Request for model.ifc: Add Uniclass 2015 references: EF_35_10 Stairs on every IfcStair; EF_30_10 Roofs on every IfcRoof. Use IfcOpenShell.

First a look at what the model holds.

```python
import ifcopenshell

model = ifcopenshell.open("model.ifc")
print(model.schema)
print("classifications:", [c.Name for c in model.by_type("IfcClassification")])
for ifc_class in ("IfcDoor", "IfcRoof", "IfcStair", "IfcWall", "IfcWindow"):
    print(ifc_class, len(model.by_type(ifc_class)))
```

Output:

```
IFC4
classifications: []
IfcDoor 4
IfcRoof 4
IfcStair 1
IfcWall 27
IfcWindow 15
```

```python
import ifcopenshell
import ifcopenshell.api.classification

model = ifcopenshell.open("model.ifc")

system = ifcopenshell.api.classification.add_classification(model, classification="Uniclass 2015")

codes = {
    "IfcStair": ("EF_35_10", "Stairs"),
    "IfcRoof": ("EF_30_10", "Roofs"),
}
for ifc_class, (code, name) in codes.items():
    products = model.by_type(ifc_class)
    ifcopenshell.api.classification.add_reference(
        model, products=products, classification=system, identification=code, name=name
    )
    print(code, len(products))

model.write("model_rev.ifc")
```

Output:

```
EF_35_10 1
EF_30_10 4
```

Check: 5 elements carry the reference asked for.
